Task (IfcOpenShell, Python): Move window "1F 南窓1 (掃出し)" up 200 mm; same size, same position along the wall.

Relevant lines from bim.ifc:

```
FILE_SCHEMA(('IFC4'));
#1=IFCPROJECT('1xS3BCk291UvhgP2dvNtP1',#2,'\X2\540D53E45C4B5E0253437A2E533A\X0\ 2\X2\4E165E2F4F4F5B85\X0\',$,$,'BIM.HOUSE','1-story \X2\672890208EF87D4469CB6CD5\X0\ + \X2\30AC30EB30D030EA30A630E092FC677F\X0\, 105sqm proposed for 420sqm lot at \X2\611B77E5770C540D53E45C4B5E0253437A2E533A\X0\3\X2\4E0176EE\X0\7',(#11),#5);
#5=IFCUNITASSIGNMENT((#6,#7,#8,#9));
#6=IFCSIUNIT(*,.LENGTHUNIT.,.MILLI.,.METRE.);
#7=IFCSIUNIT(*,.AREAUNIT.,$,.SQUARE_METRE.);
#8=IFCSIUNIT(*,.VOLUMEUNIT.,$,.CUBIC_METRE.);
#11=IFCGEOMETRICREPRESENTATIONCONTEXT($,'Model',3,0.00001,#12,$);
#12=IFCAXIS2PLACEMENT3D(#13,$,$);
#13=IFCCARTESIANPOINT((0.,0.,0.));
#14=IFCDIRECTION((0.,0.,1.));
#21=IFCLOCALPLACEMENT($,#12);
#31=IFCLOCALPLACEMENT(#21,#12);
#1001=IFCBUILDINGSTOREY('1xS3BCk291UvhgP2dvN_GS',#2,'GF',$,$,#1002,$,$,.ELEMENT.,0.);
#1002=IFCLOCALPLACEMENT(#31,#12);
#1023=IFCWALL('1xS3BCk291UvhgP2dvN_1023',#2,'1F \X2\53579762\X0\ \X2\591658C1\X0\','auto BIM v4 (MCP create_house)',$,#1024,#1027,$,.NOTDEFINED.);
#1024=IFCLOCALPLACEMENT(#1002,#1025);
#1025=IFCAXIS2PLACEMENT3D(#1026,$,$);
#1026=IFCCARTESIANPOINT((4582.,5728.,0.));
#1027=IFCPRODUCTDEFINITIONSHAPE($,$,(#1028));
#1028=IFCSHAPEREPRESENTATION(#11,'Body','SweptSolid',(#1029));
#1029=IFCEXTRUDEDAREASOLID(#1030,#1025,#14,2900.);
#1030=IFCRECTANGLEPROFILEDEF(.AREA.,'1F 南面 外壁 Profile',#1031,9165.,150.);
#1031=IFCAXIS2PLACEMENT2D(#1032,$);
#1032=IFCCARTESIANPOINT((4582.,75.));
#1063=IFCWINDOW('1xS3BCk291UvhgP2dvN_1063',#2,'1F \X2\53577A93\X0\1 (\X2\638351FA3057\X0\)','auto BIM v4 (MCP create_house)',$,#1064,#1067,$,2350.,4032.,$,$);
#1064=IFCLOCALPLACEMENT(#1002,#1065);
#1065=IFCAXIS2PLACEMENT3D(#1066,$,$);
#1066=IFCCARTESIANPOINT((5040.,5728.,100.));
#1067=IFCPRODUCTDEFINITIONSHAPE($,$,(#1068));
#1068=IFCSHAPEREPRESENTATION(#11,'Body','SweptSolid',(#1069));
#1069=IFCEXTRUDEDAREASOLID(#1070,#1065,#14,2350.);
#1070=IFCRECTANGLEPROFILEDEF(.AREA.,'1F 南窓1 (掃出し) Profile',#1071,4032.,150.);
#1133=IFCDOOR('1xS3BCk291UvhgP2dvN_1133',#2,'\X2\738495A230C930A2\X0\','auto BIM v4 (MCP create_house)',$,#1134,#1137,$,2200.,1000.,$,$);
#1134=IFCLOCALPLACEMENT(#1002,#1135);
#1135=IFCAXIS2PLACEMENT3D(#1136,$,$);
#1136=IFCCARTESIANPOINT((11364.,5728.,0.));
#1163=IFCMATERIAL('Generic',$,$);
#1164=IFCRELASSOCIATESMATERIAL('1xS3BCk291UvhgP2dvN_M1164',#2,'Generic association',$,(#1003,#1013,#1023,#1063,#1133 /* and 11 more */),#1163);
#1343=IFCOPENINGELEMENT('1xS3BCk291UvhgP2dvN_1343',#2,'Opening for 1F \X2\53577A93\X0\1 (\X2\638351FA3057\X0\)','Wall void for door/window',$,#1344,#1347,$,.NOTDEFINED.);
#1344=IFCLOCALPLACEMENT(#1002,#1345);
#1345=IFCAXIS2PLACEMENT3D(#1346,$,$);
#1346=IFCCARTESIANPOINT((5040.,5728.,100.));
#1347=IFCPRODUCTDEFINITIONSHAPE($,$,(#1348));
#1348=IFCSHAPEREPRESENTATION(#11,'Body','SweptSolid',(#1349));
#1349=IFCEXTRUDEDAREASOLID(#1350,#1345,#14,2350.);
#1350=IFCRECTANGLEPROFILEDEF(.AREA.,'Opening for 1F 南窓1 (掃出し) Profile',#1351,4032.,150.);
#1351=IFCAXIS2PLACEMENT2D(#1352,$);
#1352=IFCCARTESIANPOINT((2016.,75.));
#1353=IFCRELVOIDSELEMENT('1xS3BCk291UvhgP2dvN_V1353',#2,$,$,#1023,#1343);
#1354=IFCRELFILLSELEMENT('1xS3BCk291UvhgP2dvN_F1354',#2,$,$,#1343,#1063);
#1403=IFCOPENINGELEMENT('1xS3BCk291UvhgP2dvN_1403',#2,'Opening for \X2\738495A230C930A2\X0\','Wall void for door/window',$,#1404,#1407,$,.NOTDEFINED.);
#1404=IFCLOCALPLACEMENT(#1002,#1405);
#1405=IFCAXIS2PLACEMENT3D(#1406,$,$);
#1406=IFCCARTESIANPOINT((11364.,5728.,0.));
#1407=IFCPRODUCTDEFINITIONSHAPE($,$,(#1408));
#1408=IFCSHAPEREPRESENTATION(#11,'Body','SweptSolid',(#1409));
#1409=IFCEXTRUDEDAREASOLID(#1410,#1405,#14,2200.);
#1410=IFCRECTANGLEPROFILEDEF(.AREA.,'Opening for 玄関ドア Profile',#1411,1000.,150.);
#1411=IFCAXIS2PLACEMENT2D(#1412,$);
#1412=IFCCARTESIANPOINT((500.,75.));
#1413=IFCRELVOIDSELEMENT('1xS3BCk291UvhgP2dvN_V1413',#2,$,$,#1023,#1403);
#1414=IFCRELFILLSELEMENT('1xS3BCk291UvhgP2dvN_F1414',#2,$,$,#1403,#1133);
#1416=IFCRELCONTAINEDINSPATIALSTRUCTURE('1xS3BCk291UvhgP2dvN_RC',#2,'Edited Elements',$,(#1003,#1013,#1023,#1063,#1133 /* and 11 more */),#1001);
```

```python
import numpy as np
import ifcopenshell
import ifcopenshell.api.geometry
import ifcopenshell.util.placement
import ifcopenshell.util.unit

model = ifcopenshell.open("bim.ifc")
unit_scale = ifcopenshell.util.unit.calculate_unit_scale(model)

window = model.by_guid("1xS3BCk291UvhgP2dvN_1063")
opening = window.FillsVoids[0].RelatingOpeningElement
dz = 200.0

shift = np.array([0.0, 0.0, dz])
# The window is not placed relative to its opening, so move both.
for product in (opening, window):
    matrix = ifcopenshell.util.placement.get_local_placement(product.ObjectPlacement)
    matrix[:3, 3] += shift
    ifcopenshell.api.geometry.edit_object_placement(model, product=product, matrix=matrix, is_si=False)

print(f"moved by {dz * unit_scale:+.3f} m")

model.write("bim_v2.ifc")
```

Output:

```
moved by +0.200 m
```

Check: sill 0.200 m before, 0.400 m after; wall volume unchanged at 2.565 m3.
